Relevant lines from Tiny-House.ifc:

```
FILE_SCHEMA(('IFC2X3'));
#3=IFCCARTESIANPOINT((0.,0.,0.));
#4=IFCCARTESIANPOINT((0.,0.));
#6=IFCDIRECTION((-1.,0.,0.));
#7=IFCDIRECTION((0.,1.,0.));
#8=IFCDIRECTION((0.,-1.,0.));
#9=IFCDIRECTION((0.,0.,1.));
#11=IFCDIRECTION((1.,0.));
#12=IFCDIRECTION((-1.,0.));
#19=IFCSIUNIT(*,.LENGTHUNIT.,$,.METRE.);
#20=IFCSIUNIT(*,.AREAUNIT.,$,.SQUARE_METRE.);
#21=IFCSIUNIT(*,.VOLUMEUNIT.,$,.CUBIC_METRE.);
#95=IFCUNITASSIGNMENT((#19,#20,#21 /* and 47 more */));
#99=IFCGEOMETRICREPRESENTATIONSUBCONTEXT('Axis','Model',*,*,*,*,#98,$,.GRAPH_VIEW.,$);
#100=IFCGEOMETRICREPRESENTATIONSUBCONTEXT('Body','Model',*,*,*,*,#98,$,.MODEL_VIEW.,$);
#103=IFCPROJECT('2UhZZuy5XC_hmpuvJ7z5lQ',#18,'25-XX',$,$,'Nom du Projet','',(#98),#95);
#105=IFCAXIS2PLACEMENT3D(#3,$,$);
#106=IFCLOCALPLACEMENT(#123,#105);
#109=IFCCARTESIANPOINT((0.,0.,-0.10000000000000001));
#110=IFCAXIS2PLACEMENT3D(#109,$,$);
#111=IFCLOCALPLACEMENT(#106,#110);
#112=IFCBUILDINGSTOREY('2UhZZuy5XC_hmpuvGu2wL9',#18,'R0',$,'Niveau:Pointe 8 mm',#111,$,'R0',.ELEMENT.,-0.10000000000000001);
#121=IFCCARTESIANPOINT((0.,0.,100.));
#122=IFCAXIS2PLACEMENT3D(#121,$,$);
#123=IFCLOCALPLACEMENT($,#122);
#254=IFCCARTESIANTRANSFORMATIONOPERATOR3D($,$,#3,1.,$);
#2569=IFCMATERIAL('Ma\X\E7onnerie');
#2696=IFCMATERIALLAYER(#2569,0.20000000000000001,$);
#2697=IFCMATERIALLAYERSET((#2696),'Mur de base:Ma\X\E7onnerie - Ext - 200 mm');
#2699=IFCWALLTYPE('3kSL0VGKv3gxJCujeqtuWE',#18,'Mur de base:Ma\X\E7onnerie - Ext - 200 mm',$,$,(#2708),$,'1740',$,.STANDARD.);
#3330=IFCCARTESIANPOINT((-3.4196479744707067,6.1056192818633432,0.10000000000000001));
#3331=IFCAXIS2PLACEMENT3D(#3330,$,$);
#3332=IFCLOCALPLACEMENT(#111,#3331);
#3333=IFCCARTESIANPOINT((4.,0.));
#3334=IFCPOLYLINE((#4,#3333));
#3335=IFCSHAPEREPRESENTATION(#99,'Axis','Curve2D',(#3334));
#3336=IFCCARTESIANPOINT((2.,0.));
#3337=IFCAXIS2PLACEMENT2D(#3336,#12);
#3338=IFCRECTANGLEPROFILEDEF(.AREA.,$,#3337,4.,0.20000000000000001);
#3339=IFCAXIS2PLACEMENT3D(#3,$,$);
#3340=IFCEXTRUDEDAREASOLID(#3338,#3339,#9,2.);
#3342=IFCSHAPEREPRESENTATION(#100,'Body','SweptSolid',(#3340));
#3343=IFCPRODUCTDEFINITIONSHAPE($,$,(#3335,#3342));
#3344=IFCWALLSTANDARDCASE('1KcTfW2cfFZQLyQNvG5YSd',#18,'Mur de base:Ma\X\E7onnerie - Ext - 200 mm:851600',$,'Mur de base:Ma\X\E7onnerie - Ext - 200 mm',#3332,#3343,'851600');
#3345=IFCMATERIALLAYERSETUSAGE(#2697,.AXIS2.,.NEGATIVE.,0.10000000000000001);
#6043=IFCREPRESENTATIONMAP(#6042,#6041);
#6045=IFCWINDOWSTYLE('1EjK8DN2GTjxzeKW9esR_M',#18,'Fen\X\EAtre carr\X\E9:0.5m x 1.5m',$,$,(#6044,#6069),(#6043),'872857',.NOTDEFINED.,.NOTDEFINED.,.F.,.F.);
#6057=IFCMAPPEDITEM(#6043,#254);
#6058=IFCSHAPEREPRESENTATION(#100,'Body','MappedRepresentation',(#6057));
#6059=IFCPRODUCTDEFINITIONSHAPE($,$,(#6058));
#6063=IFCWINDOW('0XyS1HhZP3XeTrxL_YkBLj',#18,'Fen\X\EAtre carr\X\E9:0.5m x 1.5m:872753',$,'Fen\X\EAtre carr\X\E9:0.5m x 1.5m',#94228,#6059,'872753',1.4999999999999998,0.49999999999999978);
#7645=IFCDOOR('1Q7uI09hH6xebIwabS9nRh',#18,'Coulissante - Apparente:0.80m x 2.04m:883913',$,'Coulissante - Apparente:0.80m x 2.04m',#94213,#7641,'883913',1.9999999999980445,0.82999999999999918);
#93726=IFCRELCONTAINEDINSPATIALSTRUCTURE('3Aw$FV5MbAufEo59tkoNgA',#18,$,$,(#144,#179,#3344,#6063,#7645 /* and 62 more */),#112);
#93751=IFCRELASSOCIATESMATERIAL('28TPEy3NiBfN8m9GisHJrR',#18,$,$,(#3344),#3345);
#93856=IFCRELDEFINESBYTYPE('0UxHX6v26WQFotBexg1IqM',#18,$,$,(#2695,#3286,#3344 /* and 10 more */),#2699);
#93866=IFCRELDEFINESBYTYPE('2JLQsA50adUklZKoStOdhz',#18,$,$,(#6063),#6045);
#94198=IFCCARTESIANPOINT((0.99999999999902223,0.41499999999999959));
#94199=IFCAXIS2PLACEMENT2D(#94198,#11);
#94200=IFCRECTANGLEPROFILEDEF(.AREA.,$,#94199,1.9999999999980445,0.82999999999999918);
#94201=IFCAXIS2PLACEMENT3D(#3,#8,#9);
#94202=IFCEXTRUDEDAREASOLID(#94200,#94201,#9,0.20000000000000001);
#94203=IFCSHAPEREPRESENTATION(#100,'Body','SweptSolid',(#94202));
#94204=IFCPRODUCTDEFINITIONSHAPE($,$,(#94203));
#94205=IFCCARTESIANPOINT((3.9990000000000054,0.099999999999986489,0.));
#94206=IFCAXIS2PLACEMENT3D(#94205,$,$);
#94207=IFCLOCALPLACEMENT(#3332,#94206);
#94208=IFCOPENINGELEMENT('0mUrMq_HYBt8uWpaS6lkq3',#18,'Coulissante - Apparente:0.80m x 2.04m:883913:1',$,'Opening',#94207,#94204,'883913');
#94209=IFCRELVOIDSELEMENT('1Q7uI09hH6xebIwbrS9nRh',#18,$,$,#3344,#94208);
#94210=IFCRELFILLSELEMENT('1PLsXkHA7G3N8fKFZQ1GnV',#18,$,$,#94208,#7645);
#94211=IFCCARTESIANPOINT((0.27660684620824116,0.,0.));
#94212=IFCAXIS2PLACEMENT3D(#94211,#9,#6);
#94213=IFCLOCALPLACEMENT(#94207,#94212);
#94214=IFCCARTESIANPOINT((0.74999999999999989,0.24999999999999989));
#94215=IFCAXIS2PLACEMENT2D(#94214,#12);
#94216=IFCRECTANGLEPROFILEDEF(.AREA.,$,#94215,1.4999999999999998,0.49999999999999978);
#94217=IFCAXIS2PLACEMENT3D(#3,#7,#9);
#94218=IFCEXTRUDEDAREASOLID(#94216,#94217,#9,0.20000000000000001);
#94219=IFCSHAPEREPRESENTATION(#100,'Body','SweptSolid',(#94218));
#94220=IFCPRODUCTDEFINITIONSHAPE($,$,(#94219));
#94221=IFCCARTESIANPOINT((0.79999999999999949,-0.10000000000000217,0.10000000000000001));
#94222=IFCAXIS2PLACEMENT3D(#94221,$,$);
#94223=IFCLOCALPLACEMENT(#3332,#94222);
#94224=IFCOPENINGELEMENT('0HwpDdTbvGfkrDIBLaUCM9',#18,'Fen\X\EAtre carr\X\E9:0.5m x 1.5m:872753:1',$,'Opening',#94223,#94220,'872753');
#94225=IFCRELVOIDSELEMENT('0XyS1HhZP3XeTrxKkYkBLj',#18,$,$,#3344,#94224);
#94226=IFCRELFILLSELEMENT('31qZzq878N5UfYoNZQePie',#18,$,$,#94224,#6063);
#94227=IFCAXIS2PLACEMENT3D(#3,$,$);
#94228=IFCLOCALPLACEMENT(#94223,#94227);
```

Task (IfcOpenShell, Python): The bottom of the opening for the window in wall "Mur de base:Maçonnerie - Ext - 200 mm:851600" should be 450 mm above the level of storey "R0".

```python
import numpy as np
import ifcopenshell
import ifcopenshell.api.geometry
import ifcopenshell.geom
import ifcopenshell.util.element
import ifcopenshell.util.placement
import ifcopenshell.util.shape
import ifcopenshell.util.unit

model = ifcopenshell.open("Tiny-House.ifc")
unit_scale = ifcopenshell.util.unit.calculate_unit_scale(model)

window = model.by_guid("0XyS1HhZP3XeTrxL_YkBLj")
opening = window.FillsVoids[0].RelatingOpeningElement
storey = ifcopenshell.util.element.get_container(window, ifc_class="IfcBuildingStorey")
level = ifcopenshell.util.placement.get_local_placement(storey.ObjectPlacement)[2, 3]

# The opening's origin need not be at the sill, so measure its lowest point.
shape = ifcopenshell.geom.create_shape(ifcopenshell.geom.settings(), opening)
bottom = ifcopenshell.util.shape.get_shape_bottom_elevation(shape, shape.geometry) / unit_scale
dz = level + 0.45 - bottom

shift = np.array([0.0, 0.0, dz])
# The window is placed relative to its opening, so it follows when the opening moves.
matrix = ifcopenshell.util.placement.get_local_placement(opening.ObjectPlacement)
matrix[:3, 3] += shift
ifcopenshell.api.geometry.edit_object_placement(
    model, product=opening, matrix=matrix, is_si=False, should_transform_children=True
)

print(f"moved by {dz * unit_scale:+.3f} m")

model.write("Tiny-House_rev.ifc")
```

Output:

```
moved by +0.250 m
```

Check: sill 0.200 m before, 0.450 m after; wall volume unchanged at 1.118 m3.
